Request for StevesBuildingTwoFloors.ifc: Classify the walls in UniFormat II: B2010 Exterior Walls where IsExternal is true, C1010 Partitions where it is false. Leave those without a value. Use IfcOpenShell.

First a look at what the model holds.

```python
import ifcopenshell
import ifcopenshell.util.element

model = ifcopenshell.open("StevesBuildingTwoFloors.ifc")
print(model.schema)
print("classifications:", [c.Name for c in model.by_type("IfcClassification")])
values = [ifcopenshell.util.element.get_pset(e, "Pset_WallCommon", "IsExternal") for e in model.by_type("IfcWall")]
for value in (True, False, None):
    print("IsExternal", value, values.count(value))
```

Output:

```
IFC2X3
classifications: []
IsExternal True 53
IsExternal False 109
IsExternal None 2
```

```python
import ifcopenshell
import ifcopenshell.api.classification
import ifcopenshell.util.element

model = ifcopenshell.open("StevesBuildingTwoFloors.ifc")

# IFC2X3 requires Source and Edition and has no link from the project to the system.
system = model.create_entity("IfcClassification", Source="ASTM", Edition="E1557", Name="UniFormat II")

walls = model.by_type("IfcWall")
external = {e: ifcopenshell.util.element.get_pset(e, "Pset_WallCommon", "IsExternal") for e in walls}
for flag, code, name in ((True, "B2010", "Exterior Walls"), (False, "C1010", "Partitions")):
    products = [e for e in walls if external[e] is flag]
    ifcopenshell.api.classification.add_reference(
        model, products=products, classification=system, identification=code, name=name
    )
    print(code, len(products))

model.write("StevesBuildingTwoFloors_rev.ifc")
```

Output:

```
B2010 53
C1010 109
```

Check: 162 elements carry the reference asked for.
